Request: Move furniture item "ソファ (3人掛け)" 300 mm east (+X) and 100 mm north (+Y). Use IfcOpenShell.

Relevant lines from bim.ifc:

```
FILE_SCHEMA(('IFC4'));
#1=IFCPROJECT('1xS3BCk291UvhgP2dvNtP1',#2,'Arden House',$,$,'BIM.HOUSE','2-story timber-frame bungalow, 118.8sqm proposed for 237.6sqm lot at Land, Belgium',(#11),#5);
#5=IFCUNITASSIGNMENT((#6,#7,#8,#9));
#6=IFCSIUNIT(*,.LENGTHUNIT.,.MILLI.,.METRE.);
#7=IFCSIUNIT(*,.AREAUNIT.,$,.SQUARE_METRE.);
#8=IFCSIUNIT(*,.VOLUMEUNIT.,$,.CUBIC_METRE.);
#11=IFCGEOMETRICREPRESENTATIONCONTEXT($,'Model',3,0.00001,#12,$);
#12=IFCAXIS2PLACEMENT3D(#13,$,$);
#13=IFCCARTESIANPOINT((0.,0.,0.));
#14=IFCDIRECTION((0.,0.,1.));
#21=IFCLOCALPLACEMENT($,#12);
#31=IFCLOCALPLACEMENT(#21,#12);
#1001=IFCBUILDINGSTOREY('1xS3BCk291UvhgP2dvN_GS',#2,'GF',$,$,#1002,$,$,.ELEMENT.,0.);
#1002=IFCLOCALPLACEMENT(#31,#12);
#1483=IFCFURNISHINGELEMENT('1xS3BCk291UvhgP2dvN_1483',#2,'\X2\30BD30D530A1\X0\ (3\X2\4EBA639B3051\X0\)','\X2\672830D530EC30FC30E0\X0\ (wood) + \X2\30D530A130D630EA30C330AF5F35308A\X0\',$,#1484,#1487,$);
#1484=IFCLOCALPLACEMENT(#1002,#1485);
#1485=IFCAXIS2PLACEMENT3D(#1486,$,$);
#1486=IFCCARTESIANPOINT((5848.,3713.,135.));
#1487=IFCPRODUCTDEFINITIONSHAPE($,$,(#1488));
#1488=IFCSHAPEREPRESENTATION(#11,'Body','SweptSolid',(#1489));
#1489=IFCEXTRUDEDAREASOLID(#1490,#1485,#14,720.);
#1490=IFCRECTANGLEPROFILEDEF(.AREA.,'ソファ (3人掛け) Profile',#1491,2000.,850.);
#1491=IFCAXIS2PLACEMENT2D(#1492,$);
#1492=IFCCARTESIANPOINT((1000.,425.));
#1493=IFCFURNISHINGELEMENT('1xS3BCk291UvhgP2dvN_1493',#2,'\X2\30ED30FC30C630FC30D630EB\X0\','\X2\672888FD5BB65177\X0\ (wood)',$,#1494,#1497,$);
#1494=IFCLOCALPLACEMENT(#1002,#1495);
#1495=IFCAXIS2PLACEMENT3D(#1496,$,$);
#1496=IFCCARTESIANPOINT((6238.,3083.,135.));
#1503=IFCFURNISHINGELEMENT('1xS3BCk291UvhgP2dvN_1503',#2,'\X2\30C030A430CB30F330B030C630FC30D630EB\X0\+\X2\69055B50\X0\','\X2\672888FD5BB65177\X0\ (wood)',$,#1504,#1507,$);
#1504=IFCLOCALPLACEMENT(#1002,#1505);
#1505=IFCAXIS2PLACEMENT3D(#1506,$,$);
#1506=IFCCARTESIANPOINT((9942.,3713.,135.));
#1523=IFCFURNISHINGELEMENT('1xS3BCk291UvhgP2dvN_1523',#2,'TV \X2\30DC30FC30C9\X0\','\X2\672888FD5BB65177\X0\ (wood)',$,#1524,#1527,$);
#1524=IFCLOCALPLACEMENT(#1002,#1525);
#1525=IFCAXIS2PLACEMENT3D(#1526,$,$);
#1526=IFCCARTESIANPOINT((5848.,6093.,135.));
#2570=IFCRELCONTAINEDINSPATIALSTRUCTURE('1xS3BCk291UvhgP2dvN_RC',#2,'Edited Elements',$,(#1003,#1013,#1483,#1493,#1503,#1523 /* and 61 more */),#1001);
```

```python
import ifcopenshell
import ifcopenshell.api.geometry
import ifcopenshell.util.placement
import ifcopenshell.util.unit

model = ifcopenshell.open("bim.ifc")
unit_scale = ifcopenshell.util.unit.calculate_unit_scale(model)

item = model.by_id(1483)
matrix = ifcopenshell.util.placement.get_local_placement(item.ObjectPlacement)
matrix[0, 3] += 0.3 / unit_scale
matrix[1, 3] += 0.1 / unit_scale
ifcopenshell.api.geometry.edit_object_placement(model, product=item, matrix=matrix, is_si=False)

print(ifcopenshell.util.placement.get_local_placement(item.ObjectPlacement).round(3) + 0.0)

model.write("bim_updated.ifc")
```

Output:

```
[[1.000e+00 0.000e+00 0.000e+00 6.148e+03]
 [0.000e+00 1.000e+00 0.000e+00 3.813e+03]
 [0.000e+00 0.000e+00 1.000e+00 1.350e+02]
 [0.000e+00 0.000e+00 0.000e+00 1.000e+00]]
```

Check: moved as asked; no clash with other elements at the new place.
